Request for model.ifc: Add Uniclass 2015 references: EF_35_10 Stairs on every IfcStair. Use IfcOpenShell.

First a look at what the model holds.

```python
import ifcopenshell

model = ifcopenshell.open("model.ifc")
print(model.schema)
print("classifications:", [c.Name for c in model.by_type("IfcClassification")])
for ifc_class in ("IfcDoor", "IfcRoof", "IfcStair", "IfcWall", "IfcWindow"):
    print(ifc_class, len(model.by_type(ifc_class)))
```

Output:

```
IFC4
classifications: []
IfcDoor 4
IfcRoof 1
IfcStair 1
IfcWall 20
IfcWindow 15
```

```python
import ifcopenshell
import ifcopenshell.api.classification

model = ifcopenshell.open("model.ifc")

system = ifcopenshell.api.classification.add_classification(model, classification="Uniclass 2015")

codes = {
    "IfcStair": ("EF_35_10", "Stairs"),
}
for ifc_class, (code, name) in codes.items():
    products = model.by_type(ifc_class)
    ifcopenshell.api.classification.add_reference(
        model, products=products, classification=system, identification=code, name=name
    )
    print(code, len(products))

model.write("model_rev.ifc")
```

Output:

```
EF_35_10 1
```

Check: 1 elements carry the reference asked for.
